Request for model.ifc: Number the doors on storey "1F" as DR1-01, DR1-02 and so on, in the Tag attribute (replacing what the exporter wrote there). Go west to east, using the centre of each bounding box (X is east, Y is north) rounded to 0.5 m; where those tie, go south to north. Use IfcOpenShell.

First a look at what the model holds.

```python
import ifcopenshell
import ifcopenshell.util.element
import ifcopenshell.util.placement

model = ifcopenshell.open("model.ifc")
print(model.schema)
storey = next(s for s in model.by_type("IfcBuildingStorey") if s.Name == "1F")
doors = [e for e in ifcopenshell.util.element.get_decomposition(storey) if e.is_a("IfcDoor")]
for e in sorted(doors, key=lambda e: e.id()):
    origin = ifcopenshell.util.placement.get_local_placement(e.ObjectPlacement)[:3, 3]
    print(e.id(), e.Tag, e.Name, origin.round(2) + 0.0, sep=" | ")
```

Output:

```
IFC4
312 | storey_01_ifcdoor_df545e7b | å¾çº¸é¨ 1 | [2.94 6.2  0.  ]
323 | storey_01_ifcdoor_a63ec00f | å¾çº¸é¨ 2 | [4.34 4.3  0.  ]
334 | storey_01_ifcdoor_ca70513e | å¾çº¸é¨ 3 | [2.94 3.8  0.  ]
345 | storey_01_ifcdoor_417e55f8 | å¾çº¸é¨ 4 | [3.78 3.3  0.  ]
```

```python
import ifcopenshell
import ifcopenshell.geom
import ifcopenshell.util.element
import ifcopenshell.util.shape

model = ifcopenshell.open("model.ifc")
settings = ifcopenshell.geom.settings()
settings.set("use-world-coords", True)


def centre(element):
    shape = ifcopenshell.geom.create_shape(settings, element)
    return ifcopenshell.util.shape.get_bbox_centroid(shape.geometry)


storey = next(s for s in model.by_type("IfcBuildingStorey") if s.Name == "1F")
doors = [e for e in ifcopenshell.util.element.get_decomposition(storey) if e.is_a("IfcDoor")]

# Insertion points can sit at a corner or the storey origin, so sort by the geometry (in metres).
centres = {e: centre(e) for e in doors}
doors.sort(key=lambda e: (round(centres[e][0] / 0.5), centres[e][1]))

for i, e in enumerate(doors, start=1):
    number = f"DR1-{i:02d}"
    e.Tag = number
    print(e.id(), number)

model.write("model-out.ifc")
```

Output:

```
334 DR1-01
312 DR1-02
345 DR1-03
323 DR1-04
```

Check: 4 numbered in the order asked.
